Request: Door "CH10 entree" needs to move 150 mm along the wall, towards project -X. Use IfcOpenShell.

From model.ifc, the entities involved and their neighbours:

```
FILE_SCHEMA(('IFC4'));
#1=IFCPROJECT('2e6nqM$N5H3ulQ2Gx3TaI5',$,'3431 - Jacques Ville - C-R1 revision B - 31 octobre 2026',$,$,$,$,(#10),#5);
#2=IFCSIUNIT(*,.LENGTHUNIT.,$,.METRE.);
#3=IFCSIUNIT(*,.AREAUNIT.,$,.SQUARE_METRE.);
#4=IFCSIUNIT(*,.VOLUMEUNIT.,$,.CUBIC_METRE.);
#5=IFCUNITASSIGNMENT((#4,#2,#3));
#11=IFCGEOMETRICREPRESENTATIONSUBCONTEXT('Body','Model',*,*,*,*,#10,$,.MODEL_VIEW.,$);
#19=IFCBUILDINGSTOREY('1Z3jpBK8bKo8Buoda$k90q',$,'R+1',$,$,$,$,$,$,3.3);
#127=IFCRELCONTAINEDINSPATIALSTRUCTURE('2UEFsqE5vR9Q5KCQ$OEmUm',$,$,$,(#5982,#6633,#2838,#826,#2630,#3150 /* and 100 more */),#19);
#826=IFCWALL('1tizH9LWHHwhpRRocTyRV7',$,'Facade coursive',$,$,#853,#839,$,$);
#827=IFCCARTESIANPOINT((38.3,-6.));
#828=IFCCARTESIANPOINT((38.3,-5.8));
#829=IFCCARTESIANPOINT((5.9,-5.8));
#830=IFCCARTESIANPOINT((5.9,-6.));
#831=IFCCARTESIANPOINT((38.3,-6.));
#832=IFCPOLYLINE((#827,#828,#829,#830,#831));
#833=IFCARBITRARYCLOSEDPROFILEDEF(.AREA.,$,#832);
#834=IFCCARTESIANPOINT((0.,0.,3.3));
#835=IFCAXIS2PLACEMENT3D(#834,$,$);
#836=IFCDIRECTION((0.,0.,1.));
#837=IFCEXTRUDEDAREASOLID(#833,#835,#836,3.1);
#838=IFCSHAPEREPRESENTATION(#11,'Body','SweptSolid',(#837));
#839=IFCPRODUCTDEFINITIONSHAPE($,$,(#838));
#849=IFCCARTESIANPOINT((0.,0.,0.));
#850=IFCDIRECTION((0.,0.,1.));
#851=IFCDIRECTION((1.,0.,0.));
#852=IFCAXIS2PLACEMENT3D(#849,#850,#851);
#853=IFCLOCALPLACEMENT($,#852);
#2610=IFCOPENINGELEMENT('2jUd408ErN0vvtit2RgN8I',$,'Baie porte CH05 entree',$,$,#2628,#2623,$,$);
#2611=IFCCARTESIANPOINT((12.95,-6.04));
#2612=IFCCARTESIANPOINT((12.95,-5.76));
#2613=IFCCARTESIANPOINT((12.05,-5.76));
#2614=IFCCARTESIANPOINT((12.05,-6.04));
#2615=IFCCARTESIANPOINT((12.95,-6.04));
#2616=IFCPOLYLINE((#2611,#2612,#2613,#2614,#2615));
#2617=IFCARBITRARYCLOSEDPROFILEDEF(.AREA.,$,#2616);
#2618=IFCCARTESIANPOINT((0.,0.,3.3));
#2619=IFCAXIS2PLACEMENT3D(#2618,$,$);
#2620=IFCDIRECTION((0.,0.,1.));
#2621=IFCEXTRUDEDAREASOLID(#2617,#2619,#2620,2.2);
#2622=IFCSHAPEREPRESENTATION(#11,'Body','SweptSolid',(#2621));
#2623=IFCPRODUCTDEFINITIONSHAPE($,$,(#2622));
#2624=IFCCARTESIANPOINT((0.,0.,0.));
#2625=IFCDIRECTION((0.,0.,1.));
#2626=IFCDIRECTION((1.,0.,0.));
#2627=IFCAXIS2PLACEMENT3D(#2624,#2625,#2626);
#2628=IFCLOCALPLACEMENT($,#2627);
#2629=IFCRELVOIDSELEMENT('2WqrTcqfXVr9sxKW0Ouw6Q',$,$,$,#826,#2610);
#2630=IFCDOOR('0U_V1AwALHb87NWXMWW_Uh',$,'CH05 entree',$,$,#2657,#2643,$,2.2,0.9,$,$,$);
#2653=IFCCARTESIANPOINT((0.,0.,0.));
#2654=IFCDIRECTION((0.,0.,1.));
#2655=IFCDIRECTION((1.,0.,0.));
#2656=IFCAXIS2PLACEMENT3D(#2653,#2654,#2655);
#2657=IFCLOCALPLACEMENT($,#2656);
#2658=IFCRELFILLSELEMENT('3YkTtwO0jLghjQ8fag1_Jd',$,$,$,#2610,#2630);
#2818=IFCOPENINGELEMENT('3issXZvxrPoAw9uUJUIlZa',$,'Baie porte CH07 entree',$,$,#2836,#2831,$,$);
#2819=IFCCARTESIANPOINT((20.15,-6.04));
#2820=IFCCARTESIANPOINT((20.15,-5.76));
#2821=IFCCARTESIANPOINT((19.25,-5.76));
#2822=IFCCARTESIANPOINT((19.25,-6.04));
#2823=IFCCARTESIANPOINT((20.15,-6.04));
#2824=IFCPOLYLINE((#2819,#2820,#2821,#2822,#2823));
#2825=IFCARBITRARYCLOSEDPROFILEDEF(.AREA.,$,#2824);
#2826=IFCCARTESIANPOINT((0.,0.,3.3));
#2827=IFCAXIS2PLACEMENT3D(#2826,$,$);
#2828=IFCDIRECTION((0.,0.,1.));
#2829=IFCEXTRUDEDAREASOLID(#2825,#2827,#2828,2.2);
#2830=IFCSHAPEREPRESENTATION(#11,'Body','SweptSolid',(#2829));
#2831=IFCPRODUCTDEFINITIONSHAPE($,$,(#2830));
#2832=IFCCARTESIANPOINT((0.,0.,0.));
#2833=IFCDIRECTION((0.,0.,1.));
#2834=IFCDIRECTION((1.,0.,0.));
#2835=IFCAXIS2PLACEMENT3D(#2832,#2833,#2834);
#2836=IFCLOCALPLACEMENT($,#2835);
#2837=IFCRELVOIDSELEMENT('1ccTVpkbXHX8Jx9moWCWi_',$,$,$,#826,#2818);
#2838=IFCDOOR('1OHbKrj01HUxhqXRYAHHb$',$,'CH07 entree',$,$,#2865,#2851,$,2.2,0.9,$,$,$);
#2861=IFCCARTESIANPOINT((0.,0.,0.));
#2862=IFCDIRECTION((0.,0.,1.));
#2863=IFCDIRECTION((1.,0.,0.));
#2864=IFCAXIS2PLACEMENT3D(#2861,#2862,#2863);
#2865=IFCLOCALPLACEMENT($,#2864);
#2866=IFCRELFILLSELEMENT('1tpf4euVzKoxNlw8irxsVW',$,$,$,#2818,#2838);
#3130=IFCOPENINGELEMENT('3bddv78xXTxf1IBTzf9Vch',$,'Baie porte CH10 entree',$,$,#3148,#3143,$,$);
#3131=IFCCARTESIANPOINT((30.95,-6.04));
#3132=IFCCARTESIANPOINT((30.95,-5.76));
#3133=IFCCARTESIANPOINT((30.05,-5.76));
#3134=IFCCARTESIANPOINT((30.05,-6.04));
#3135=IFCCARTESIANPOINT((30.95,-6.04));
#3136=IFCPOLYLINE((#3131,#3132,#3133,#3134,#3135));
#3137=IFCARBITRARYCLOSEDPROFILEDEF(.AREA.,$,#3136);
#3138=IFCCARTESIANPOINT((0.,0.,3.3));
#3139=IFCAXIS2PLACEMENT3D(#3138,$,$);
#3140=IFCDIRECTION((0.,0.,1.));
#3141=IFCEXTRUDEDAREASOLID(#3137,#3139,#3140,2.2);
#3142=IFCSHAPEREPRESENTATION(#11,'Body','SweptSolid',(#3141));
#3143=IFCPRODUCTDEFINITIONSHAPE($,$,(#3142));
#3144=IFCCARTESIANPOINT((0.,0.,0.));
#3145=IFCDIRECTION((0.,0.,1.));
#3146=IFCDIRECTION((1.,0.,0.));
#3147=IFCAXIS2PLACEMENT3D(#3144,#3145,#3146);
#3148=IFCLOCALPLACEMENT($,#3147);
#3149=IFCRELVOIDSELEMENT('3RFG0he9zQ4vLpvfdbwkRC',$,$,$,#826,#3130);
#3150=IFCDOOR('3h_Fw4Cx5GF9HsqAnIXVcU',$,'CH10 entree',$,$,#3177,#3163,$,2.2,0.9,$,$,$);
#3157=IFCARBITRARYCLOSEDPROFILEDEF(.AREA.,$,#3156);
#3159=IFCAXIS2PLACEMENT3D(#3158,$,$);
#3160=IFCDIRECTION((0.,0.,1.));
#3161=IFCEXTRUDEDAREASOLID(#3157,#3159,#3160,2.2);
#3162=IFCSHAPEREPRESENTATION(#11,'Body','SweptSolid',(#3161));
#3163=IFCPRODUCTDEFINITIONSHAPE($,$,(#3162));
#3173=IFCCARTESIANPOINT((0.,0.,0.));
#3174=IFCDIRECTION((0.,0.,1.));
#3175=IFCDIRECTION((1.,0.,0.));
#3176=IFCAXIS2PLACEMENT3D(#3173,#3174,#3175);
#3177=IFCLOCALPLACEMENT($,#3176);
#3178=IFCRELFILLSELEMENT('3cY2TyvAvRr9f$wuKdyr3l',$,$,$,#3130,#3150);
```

```python
import ifcopenshell
import ifcopenshell.api.geometry
import ifcopenshell.util.placement

model = ifcopenshell.open("model.ifc")

door = model.by_guid("3h_Fw4Cx5GF9HsqAnIXVcU")
opening = door.FillsVoids[0].RelatingOpeningElement
wall = opening.VoidsElements[0].RelatingBuildingElement

wall_matrix = ifcopenshell.util.placement.get_local_placement(wall.ObjectPlacement)
shift = wall_matrix[:3, 0] * -0.15
before = ifcopenshell.util.placement.get_local_placement(door.ObjectPlacement)[:3, 3].copy()

# The door is not placed relative to its opening, so move both.
for product in (opening, door):
    matrix = ifcopenshell.util.placement.get_local_placement(product.ObjectPlacement)
    matrix[:3, 3] += shift
    ifcopenshell.api.geometry.edit_object_placement(model, product=product, matrix=matrix, is_si=False)

after = ifcopenshell.util.placement.get_local_placement(door.ObjectPlacement)[:3, 3]
print("door moved by", (after - before).round(3) + 0.0)

model.write("model-out.ifc")
```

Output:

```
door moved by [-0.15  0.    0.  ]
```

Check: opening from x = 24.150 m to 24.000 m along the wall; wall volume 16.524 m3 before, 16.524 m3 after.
